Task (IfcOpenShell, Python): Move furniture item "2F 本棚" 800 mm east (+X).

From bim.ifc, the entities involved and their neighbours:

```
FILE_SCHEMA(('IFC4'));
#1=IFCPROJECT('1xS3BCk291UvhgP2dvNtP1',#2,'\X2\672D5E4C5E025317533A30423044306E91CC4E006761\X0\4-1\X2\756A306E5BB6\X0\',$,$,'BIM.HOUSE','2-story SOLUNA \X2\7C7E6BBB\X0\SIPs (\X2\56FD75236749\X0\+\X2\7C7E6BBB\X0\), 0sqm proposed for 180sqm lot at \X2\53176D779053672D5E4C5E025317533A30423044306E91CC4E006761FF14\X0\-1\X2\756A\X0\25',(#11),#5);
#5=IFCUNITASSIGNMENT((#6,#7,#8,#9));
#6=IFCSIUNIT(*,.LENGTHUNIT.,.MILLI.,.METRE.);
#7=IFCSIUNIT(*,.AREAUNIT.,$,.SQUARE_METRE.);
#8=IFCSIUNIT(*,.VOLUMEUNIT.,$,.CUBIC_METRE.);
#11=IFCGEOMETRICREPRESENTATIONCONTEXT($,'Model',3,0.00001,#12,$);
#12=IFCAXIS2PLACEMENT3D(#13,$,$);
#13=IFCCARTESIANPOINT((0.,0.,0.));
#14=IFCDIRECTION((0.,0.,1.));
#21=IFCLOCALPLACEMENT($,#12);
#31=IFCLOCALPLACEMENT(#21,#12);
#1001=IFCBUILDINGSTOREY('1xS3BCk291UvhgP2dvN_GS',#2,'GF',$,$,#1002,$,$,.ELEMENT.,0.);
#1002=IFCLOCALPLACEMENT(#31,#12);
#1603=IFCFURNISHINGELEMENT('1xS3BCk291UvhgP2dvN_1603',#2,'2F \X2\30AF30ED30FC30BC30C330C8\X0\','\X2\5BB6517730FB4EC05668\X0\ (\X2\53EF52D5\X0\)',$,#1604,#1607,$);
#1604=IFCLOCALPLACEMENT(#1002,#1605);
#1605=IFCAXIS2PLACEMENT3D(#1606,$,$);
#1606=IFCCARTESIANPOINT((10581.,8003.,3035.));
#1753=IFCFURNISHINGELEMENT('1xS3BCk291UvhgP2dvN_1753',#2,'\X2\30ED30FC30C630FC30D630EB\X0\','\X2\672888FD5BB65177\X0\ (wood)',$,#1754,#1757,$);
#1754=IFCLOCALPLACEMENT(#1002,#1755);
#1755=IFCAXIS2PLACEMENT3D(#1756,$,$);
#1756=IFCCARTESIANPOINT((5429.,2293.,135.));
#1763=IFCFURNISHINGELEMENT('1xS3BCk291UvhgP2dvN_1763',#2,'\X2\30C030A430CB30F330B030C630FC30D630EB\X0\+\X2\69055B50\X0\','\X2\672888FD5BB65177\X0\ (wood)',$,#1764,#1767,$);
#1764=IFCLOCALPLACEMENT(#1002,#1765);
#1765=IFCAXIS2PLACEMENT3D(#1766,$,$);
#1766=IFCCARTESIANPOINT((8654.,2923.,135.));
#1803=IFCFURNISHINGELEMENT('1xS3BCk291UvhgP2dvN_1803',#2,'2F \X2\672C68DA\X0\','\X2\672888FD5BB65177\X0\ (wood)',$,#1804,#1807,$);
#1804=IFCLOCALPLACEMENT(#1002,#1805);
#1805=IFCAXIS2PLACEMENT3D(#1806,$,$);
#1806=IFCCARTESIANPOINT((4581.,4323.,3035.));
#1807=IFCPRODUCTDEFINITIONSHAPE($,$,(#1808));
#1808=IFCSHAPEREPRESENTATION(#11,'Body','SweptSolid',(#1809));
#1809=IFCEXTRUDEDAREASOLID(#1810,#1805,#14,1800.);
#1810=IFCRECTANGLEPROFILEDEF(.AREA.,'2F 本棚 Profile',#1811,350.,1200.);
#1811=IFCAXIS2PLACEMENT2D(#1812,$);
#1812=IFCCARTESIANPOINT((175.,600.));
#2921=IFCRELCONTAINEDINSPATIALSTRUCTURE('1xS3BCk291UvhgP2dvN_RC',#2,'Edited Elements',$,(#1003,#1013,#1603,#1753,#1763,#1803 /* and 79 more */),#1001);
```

```python
import ifcopenshell
import ifcopenshell.api.geometry
import ifcopenshell.util.placement

model = ifcopenshell.open("bim.ifc")

item = model.by_guid("1xS3BCk291UvhgP2dvN_1803")
matrix = ifcopenshell.util.placement.get_local_placement(item.ObjectPlacement)
matrix[0, 3] += 800.0
ifcopenshell.api.geometry.edit_object_placement(model, product=item, matrix=matrix, is_si=False)

print(ifcopenshell.util.placement.get_local_placement(item.ObjectPlacement).round(3) + 0.0)

model.write("bim-out.ifc")
```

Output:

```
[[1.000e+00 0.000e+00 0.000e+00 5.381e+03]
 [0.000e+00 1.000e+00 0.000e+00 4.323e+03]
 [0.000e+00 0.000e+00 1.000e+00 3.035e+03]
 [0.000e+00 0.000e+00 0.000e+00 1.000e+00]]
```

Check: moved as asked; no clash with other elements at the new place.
